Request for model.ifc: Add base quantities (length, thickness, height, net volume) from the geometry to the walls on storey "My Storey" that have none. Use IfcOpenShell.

First a look at what the model holds.

```python
import ifcopenshell
import ifcopenshell.util.element
import ifcopenshell.util.unit

model = ifcopenshell.open("model.ifc")
print(model.schema)
for unit_type in ("LENGTHUNIT", "AREAUNIT", "VOLUMEUNIT"):
    print(unit_type, ifcopenshell.util.unit.calculate_unit_scale(model, unit_type))
storey = next(s for s in model.by_type("IfcBuildingStorey") if s.Name == "My Storey")
walls = [e for e in ifcopenshell.util.element.get_decomposition(storey) if e.is_a("IfcWall")]
for e in sorted(walls, key=lambda e: e.id()):
    print(e.id(), e.is_a(), e.Name, list(ifcopenshell.util.element.get_psets(e, qtos_only=True)), sep=" | ")
```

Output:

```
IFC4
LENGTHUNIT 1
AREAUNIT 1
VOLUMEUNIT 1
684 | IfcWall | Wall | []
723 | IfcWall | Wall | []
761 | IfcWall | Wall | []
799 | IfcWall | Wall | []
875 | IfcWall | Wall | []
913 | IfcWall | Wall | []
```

```python
import ifcopenshell
import ifcopenshell.api.pset
import ifcopenshell.geom
import ifcopenshell.util.element
import ifcopenshell.util.shape
import ifcopenshell.util.unit

model = ifcopenshell.open("model.ifc")
unit_scale = ifcopenshell.util.unit.calculate_unit_scale(model)
volume_scale = ifcopenshell.util.unit.calculate_unit_scale(model, "VOLUMEUNIT")
settings = ifcopenshell.geom.settings()

storey = next(s for s in model.by_type("IfcBuildingStorey") if s.Name == "My Storey")
walls = [e for e in ifcopenshell.util.element.get_decomposition(storey) if e.is_a("IfcWall")]

for e in sorted(walls, key=lambda e: e.id()):
    if ifcopenshell.util.element.get_psets(e, qtos_only=True, should_inherit=False):
        continue
    # Geometry comes back in metres, in the element's own axes.
    shape = ifcopenshell.geom.create_shape(settings, e)
    values = {
        "Length": ifcopenshell.util.shape.get_x(shape.geometry) / unit_scale,
        "Width": ifcopenshell.util.shape.get_y(shape.geometry) / unit_scale,
        "Height": ifcopenshell.util.shape.get_z(shape.geometry) / unit_scale,
        "NetVolume": ifcopenshell.util.shape.get_volume(shape.geometry) / volume_scale,
    }
    qto = ifcopenshell.api.pset.add_qto(model, product=e, name="Qto_WallBaseQuantities")
    ifcopenshell.api.pset.edit_qto(model, qto=qto, properties=values)
    print(e.id(), {k: round(v, 3) for k, v in values.items()})

model.write("model_v2.ifc")
```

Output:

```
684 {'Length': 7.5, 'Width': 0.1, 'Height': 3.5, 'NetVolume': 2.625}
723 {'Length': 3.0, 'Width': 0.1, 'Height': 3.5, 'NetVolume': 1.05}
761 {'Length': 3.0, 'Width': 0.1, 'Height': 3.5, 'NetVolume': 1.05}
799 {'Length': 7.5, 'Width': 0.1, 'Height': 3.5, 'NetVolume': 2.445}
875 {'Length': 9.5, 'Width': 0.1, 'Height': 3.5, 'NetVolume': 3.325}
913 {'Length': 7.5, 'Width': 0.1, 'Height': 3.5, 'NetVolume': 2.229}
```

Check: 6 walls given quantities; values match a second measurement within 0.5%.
